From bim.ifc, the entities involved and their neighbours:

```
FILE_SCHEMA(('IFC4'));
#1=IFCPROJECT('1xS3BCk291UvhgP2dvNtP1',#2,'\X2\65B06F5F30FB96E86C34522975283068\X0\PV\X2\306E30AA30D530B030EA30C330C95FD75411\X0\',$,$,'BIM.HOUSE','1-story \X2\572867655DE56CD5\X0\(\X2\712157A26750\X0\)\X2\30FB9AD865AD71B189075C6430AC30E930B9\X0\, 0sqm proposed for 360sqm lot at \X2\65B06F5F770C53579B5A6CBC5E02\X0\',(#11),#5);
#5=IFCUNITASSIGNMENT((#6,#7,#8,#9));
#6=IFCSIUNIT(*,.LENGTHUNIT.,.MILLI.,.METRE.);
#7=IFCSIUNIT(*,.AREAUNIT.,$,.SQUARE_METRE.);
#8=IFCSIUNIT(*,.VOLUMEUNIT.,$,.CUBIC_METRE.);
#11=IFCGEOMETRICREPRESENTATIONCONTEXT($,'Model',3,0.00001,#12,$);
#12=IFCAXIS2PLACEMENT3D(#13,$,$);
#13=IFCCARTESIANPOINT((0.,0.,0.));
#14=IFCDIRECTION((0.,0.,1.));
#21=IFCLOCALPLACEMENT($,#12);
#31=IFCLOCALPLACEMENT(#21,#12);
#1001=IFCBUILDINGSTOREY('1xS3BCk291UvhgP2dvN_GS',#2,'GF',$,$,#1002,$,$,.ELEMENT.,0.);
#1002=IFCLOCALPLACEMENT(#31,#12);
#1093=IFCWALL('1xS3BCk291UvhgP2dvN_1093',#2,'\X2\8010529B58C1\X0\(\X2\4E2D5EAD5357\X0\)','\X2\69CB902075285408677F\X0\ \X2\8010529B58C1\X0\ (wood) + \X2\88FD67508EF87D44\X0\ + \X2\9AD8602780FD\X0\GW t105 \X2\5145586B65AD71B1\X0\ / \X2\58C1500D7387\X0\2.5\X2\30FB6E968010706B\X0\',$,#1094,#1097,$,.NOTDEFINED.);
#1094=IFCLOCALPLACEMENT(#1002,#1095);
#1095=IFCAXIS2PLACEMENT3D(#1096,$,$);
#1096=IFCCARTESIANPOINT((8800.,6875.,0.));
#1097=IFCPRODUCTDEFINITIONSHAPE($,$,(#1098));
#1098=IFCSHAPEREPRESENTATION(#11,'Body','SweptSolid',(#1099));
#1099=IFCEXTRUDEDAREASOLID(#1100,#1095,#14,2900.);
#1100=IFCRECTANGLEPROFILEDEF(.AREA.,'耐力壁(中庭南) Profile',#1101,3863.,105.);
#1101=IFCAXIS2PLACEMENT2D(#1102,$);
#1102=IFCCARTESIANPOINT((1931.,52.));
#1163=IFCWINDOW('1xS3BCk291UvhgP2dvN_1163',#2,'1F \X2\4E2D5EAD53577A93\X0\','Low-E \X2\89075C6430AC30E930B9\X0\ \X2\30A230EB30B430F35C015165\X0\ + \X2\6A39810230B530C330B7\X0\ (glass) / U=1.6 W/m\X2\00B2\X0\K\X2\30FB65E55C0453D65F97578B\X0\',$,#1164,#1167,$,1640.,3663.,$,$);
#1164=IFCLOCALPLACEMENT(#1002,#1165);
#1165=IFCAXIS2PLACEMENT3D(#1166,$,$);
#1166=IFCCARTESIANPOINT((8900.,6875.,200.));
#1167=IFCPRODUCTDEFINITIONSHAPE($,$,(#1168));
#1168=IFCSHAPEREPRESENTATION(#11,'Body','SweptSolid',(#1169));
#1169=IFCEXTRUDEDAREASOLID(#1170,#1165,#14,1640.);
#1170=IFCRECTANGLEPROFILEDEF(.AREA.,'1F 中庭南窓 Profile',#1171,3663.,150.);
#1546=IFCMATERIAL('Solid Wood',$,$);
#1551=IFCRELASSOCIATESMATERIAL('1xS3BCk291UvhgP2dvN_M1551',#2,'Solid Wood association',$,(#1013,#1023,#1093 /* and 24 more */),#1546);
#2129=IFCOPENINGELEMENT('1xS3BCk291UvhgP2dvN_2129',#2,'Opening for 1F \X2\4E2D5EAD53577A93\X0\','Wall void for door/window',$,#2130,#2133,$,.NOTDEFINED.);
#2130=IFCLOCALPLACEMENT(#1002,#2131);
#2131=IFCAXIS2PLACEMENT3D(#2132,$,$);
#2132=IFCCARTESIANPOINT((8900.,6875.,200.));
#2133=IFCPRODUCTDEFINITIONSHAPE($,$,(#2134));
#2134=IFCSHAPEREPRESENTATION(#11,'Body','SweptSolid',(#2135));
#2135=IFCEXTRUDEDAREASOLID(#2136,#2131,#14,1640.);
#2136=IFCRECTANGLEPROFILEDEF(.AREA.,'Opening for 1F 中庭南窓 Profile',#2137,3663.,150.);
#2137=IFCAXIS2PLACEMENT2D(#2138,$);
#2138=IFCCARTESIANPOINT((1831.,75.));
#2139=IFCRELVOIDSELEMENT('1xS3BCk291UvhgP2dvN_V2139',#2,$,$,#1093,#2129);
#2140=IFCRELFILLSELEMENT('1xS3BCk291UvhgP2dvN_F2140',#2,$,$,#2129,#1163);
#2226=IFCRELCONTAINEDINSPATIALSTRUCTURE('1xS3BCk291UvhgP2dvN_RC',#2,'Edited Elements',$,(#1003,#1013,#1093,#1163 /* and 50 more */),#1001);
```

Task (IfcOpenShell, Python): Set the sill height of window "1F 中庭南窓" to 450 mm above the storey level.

```python
import numpy as np
import ifcopenshell
import ifcopenshell.api.geometry
import ifcopenshell.geom
import ifcopenshell.util.element
import ifcopenshell.util.placement
import ifcopenshell.util.shape
import ifcopenshell.util.unit

model = ifcopenshell.open("bim.ifc")
unit_scale = ifcopenshell.util.unit.calculate_unit_scale(model)

window = model.by_id(1163)
opening = window.FillsVoids[0].RelatingOpeningElement
storey = ifcopenshell.util.element.get_container(window, ifc_class="IfcBuildingStorey")
level = ifcopenshell.util.placement.get_local_placement(storey.ObjectPlacement)[2, 3]

# The opening's origin need not be at the sill, so measure its lowest point.
shape = ifcopenshell.geom.create_shape(ifcopenshell.geom.settings(), opening)
bottom = ifcopenshell.util.shape.get_shape_bottom_elevation(shape, shape.geometry) / unit_scale
dz = level + 0.45 / unit_scale - bottom

shift = np.array([0.0, 0.0, dz])
# The window is not placed relative to its opening, so move both.
for product in (opening, window):
    matrix = ifcopenshell.util.placement.get_local_placement(product.ObjectPlacement)
    matrix[:3, 3] += shift
    ifcopenshell.api.geometry.edit_object_placement(model, product=product, matrix=matrix, is_si=False)

print(f"moved by {dz * unit_scale:+.3f} m")

model.write("bim_updated.ifc")
```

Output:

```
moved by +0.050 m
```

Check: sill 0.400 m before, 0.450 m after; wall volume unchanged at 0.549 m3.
